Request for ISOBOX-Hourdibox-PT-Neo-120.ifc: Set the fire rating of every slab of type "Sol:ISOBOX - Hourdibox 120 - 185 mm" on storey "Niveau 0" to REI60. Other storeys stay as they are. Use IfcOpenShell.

First a look at what the model holds.

```python
import ifcopenshell
import ifcopenshell.util.element

model = ifcopenshell.open("ISOBOX-Hourdibox-PT-Neo-120.ifc")
print(model.schema)
storey = next(s for s in model.by_type("IfcBuildingStorey") if s.Name == "Niveau 0")
slabs = [e for e in ifcopenshell.util.element.get_decomposition(storey) if e.is_a("IfcSlab")]
seen = {}
for e in slabs:
    element_type = ifcopenshell.util.element.get_type(e)
    key = (element_type.Name if element_type != e and element_type else None, ifcopenshell.util.element.get_pset(e, "Pset_SlabCommon", "FireRating"))
    seen[key] = seen.get(key, 0) + 1
for (name, value), count in sorted(seen.items(), key=str):
    print(count, "x", name, "|", value)
```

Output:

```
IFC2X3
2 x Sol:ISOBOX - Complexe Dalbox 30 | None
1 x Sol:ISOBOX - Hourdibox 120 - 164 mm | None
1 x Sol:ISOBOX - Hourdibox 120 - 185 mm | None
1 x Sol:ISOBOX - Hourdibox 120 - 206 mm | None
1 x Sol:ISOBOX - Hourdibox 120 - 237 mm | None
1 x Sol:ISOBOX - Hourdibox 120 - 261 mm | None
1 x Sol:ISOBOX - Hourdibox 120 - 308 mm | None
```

```python
import ifcopenshell
import ifcopenshell.api.pset
import ifcopenshell.util.element

model = ifcopenshell.open("ISOBOX-Hourdibox-PT-Neo-120.ifc")

storey = next(s for s in model.by_type("IfcBuildingStorey") if s.Name == "Niveau 0")
slabs = [e for e in ifcopenshell.util.element.get_decomposition(storey) if e.is_a("IfcSlab")]

count = 0
for e in slabs:
    element_type = ifcopenshell.util.element.get_type(e)
    if element_type in (None, e) or element_type.Name != "Sol:ISOBOX - Hourdibox 120 - 185 mm":
        continue
    # add_pset returns the element's existing set when there is one.
    pset = ifcopenshell.api.pset.add_pset(model, product=e, name="Pset_SlabCommon")
    ifcopenshell.api.pset.edit_pset(model, pset=pset, properties={"FireRating": "REI60"})
    count += 1

print(count, "slabs updated")

model.write("ISOBOX-Hourdibox-PT-Neo-120_updated.ifc")
```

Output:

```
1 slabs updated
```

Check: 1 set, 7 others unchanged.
